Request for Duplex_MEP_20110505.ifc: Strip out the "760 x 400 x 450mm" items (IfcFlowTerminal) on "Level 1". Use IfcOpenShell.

First a look at what the model holds.

```python
import ifcopenshell
import ifcopenshell.util.element

model = ifcopenshell.open("Duplex_MEP_20110505.ifc")
print(model.schema)
storey = next(s for s in model.by_type("IfcBuildingStorey") if s.Name == "Level 1")
terminals = [e for e in ifcopenshell.util.element.get_decomposition(storey) if e.is_a("IfcFlowTerminal")]
seen = {}
for e in terminals:
    element_type = ifcopenshell.util.element.get_type(e)
    name = element_type.Name if element_type not in (None, e) else None
    seen[name] = seen.get(name, 0) + 1
for name, count in sorted(seen.items(), key=str):
    print(count, "x", name)
```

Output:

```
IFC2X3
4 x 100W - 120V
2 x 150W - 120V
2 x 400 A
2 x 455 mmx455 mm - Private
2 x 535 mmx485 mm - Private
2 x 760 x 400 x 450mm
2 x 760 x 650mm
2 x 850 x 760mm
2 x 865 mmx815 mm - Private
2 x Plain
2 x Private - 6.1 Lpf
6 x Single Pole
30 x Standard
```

```python
import ifcopenshell
import ifcopenshell.api.root
import ifcopenshell.util.element

model = ifcopenshell.open("Duplex_MEP_20110505.ifc")

storey = next(s for s in model.by_type("IfcBuildingStorey") if s.Name == "Level 1")
terminals = [e for e in ifcopenshell.util.element.get_decomposition(storey) if e.is_a("IfcFlowTerminal")]
targets = [e for e in terminals if (t := ifcopenshell.util.element.get_type(e)) not in (None, e) and t.Name == "760 x 400 x 450mm"]

for e in targets:
    ifcopenshell.api.root.remove_product(model, product=e)
print(len(targets), "removed")

model.write("Duplex_MEP_20110505_edited.ifc")
```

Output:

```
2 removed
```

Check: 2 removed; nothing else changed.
